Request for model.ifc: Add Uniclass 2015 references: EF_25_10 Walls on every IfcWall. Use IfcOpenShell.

First a look at what the model holds.

```python
import ifcopenshell

model = ifcopenshell.open("model.ifc")
print(model.schema)
print("classifications:", [c.Name for c in model.by_type("IfcClassification")])
for ifc_class in ("IfcDoor", "IfcRoof", "IfcStair", "IfcWall", "IfcWindow"):
    print(ifc_class, len(model.by_type(ifc_class)))
```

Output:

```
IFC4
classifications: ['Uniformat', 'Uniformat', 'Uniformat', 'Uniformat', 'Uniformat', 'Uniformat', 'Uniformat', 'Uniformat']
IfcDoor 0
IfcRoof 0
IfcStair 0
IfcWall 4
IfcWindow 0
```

```python
import ifcopenshell
import ifcopenshell.api.classification

model = ifcopenshell.open("model.ifc")

system = ifcopenshell.api.classification.add_classification(model, classification="Uniclass 2015")

codes = {
    "IfcWall": ("EF_25_10", "Walls"),
}
for ifc_class, (code, name) in codes.items():
    products = model.by_type(ifc_class)
    ifcopenshell.api.classification.add_reference(
        model, products=products, classification=system, identification=code, name=name
    )
    print(code, len(products))

model.write("model_edited.ifc")
```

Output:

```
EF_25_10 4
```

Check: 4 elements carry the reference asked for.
